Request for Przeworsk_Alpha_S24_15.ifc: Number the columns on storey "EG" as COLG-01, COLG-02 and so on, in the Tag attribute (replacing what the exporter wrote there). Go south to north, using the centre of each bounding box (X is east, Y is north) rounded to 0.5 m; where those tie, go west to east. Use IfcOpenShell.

First a look at what the model holds.

```python
import ifcopenshell
import ifcopenshell.util.element
import ifcopenshell.util.placement

model = ifcopenshell.open("Przeworsk_Alpha_S24_15.ifc")
print(model.schema)
storey = next(s for s in model.by_type("IfcBuildingStorey") if s.Name == "EG")
columns = [e for e in ifcopenshell.util.element.get_decomposition(storey) if e.is_a("IfcColumn")]
for e in sorted(columns, key=lambda e: e.id()):
    origin = ifcopenshell.util.placement.get_local_placement(e.ObjectPlacement)[:3, 3]
    print(e.id(), e.Tag, e.Name, origin.round(2) + 0.0, sep=" | ")
```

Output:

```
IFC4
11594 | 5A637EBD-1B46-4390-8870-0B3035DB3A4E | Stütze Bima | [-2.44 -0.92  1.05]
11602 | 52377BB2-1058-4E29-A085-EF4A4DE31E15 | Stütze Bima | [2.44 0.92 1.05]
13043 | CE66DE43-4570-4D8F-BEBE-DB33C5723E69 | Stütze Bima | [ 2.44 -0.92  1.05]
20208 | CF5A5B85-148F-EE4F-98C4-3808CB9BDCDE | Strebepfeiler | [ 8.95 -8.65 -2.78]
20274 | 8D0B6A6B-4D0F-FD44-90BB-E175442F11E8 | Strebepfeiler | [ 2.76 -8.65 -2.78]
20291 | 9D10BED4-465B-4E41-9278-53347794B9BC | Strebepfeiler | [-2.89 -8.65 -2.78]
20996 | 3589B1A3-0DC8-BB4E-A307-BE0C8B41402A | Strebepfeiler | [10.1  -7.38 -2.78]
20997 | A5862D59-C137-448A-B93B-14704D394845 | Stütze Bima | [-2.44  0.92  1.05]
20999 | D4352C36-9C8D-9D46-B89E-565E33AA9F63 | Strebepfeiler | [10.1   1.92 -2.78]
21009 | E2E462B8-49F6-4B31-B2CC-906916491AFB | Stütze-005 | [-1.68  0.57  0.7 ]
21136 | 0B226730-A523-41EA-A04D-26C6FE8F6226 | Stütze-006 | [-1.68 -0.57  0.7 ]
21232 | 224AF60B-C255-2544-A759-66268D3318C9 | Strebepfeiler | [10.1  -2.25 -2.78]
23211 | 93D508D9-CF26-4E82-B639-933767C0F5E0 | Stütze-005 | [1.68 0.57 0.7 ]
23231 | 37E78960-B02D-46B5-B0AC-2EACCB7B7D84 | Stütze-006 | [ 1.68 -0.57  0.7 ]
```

```python
import ifcopenshell
import ifcopenshell.geom
import ifcopenshell.util.element
import ifcopenshell.util.shape

model = ifcopenshell.open("Przeworsk_Alpha_S24_15.ifc")
settings = ifcopenshell.geom.settings()
settings.set("use-world-coords", True)


def centre(element):
    shape = ifcopenshell.geom.create_shape(settings, element)
    return ifcopenshell.util.shape.get_bbox_centroid(shape.geometry)


storey = next(s for s in model.by_type("IfcBuildingStorey") if s.Name == "EG")
columns = [e for e in ifcopenshell.util.element.get_decomposition(storey) if e.is_a("IfcColumn")]

# Insertion points can sit at a corner or the storey origin, so sort by the geometry (in metres).
centres = {e: centre(e) for e in columns}
columns.sort(key=lambda e: (round(centres[e][1] / 0.5), centres[e][0]))

for i, e in enumerate(columns, start=1):
    number = f"COLG-{i:02d}"
    e.Tag = number
    print(e.id(), number)

model.write("Przeworsk_Alpha_S24_15_updated.ifc")
```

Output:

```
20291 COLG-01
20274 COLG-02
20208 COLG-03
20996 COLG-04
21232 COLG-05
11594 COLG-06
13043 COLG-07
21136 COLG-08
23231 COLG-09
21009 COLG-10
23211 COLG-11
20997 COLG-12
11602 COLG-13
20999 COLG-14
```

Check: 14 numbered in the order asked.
